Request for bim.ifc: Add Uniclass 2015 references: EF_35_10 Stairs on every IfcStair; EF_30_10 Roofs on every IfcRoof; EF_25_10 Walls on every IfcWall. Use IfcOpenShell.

First a look at what the model holds.

```python
import ifcopenshell

model = ifcopenshell.open("bim.ifc")
print(model.schema)
print("classifications:", [c.Name for c in model.by_type("IfcClassification")])
for ifc_class in ("IfcDoor", "IfcRoof", "IfcStair", "IfcWall", "IfcWindow"):
    print(ifc_class, len(model.by_type(ifc_class)))
```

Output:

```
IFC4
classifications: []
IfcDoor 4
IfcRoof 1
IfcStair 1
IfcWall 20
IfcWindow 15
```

```python
import ifcopenshell
import ifcopenshell.api.classification

model = ifcopenshell.open("bim.ifc")

system = ifcopenshell.api.classification.add_classification(model, classification="Uniclass 2015")

codes = {
    "IfcStair": ("EF_35_10", "Stairs"),
    "IfcRoof": ("EF_30_10", "Roofs"),
    "IfcWall": ("EF_25_10", "Walls"),
}
for ifc_class, (code, name) in codes.items():
    products = model.by_type(ifc_class)
    ifcopenshell.api.classification.add_reference(
        model, products=products, classification=system, identification=code, name=name
    )
    print(code, len(products))

model.write("bim-out.ifc")
```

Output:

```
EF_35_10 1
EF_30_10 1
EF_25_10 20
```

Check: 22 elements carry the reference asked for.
